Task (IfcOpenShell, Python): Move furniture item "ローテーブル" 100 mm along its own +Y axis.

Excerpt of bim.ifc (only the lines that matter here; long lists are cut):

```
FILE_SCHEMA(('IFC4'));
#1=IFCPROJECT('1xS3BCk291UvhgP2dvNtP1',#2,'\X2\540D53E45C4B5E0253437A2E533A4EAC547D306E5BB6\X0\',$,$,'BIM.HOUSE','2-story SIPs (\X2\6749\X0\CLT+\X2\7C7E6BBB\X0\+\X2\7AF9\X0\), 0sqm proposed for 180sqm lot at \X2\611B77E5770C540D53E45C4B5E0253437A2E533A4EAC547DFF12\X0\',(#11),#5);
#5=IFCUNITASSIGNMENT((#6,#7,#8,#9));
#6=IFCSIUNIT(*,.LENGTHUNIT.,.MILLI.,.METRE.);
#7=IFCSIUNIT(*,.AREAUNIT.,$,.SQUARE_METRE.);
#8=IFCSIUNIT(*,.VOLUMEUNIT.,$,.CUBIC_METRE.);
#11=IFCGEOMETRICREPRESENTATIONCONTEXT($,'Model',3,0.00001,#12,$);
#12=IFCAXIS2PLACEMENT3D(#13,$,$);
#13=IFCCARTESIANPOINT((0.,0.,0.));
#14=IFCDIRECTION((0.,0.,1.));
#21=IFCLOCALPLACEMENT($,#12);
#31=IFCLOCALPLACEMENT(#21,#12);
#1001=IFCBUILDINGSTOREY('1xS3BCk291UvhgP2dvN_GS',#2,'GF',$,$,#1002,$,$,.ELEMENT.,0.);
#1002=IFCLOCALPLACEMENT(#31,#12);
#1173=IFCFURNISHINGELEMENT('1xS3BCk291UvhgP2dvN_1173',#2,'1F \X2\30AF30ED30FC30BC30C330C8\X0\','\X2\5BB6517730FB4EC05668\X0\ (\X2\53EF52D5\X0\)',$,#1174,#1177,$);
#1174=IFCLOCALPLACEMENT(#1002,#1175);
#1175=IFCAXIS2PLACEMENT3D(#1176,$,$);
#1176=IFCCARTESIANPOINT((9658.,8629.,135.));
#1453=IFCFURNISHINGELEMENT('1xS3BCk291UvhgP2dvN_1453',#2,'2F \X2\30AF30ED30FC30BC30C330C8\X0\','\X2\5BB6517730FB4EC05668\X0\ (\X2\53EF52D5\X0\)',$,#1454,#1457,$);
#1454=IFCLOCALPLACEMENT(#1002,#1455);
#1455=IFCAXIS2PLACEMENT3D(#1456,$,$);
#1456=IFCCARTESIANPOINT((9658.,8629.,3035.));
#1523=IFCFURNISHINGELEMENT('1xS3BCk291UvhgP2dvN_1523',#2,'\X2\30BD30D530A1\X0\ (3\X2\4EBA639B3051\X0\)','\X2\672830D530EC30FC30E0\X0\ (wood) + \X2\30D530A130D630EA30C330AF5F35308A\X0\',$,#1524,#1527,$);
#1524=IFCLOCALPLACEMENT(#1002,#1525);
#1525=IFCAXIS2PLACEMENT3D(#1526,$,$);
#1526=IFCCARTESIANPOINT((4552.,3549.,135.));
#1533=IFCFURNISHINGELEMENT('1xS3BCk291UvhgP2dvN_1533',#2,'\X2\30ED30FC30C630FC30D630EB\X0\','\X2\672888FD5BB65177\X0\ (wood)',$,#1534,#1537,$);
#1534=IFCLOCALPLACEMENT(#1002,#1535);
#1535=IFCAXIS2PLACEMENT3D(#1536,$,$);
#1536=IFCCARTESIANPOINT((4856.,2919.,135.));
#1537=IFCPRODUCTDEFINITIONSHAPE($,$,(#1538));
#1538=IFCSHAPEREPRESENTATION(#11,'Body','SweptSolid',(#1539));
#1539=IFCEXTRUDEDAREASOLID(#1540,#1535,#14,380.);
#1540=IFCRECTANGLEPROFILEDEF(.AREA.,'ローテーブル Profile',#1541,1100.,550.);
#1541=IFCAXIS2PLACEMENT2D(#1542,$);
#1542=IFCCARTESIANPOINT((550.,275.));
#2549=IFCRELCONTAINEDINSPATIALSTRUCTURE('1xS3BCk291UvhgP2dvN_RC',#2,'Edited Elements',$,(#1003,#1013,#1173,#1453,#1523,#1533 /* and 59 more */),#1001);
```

```python
import ifcopenshell
import ifcopenshell.api.geometry
import ifcopenshell.util.placement

model = ifcopenshell.open("bim.ifc")

item = model.by_id(1533)
matrix = ifcopenshell.util.placement.get_local_placement(item.ObjectPlacement)
matrix[:3, 3] += matrix[:3, 1] * 100.0
ifcopenshell.api.geometry.edit_object_placement(model, product=item, matrix=matrix, is_si=False)

print(ifcopenshell.util.placement.get_local_placement(item.ObjectPlacement).round(3) + 0.0)

model.write("bim_v2.ifc")
```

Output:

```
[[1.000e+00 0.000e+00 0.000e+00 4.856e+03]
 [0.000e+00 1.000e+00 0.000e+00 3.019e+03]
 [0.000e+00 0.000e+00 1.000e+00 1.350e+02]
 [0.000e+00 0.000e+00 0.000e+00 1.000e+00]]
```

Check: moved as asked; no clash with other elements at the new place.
